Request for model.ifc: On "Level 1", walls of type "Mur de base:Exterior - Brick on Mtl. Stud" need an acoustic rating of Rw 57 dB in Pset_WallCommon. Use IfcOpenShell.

First a look at what the model holds.

```python
import ifcopenshell
import ifcopenshell.util.element

model = ifcopenshell.open("model.ifc")
print(model.schema)
storey = next(s for s in model.by_type("IfcBuildingStorey") if s.Name == "Level 1")
walls = [e for e in ifcopenshell.util.element.get_decomposition(storey) if e.is_a("IfcWall")]
seen = {}
for e in walls:
    element_type = ifcopenshell.util.element.get_type(e)
    key = (element_type.Name if element_type != e and element_type else None, ifcopenshell.util.element.get_pset(e, "Pset_WallCommon", "AcousticRating"))
    seen[key] = seen.get(key, 0) + 1
for (name, value), count in sorted(seen.items(), key=str):
    print(count, "x", name, "|", value)
```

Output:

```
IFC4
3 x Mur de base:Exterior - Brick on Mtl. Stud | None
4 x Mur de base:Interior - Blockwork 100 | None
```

```python
import ifcopenshell
import ifcopenshell.api.pset
import ifcopenshell.util.element

model = ifcopenshell.open("model.ifc")

storey = next(s for s in model.by_type("IfcBuildingStorey") if s.Name == "Level 1")
walls = [e for e in ifcopenshell.util.element.get_decomposition(storey) if e.is_a("IfcWall")]

count = 0
for e in walls:
    element_type = ifcopenshell.util.element.get_type(e)
    if element_type in (None, e) or element_type.Name != "Mur de base:Exterior - Brick on Mtl. Stud":
        continue
    # add_pset returns the element's existing set when there is one.
    pset = ifcopenshell.api.pset.add_pset(model, product=e, name="Pset_WallCommon")
    ifcopenshell.api.pset.edit_pset(model, pset=pset, properties={"AcousticRating": "Rw 57 dB"})
    count += 1

print(count, "walls updated")

model.write("model_edited.ifc")
```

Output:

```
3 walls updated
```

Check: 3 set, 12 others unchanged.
